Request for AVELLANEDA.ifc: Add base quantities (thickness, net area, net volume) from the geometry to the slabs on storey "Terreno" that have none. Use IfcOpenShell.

First a look at what the model holds.

```python
import ifcopenshell
import ifcopenshell.util.element
import ifcopenshell.util.unit

model = ifcopenshell.open("AVELLANEDA.ifc")
print(model.schema)
for unit_type in ("LENGTHUNIT", "AREAUNIT", "VOLUMEUNIT"):
    print(unit_type, ifcopenshell.util.unit.calculate_unit_scale(model, unit_type))
storey = next(s for s in model.by_type("IfcBuildingStorey") if s.Name == "Terreno")
slabs = [e for e in ifcopenshell.util.element.get_decomposition(storey) if e.is_a("IfcSlab")]
for e in sorted(slabs, key=lambda e: e.id()):
    print(e.id(), e.is_a(), e.Name, list(ifcopenshell.util.element.get_psets(e, qtos_only=True)), sep=" | ")
```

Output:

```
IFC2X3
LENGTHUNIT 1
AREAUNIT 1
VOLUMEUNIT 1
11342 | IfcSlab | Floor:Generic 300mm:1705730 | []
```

```python
import ifcopenshell
import ifcopenshell.api.pset
import ifcopenshell.geom
import ifcopenshell.util.element
import ifcopenshell.util.shape
import ifcopenshell.util.unit

model = ifcopenshell.open("AVELLANEDA.ifc")
unit_scale = ifcopenshell.util.unit.calculate_unit_scale(model)
area_scale = ifcopenshell.util.unit.calculate_unit_scale(model, "AREAUNIT")
volume_scale = ifcopenshell.util.unit.calculate_unit_scale(model, "VOLUMEUNIT")
settings = ifcopenshell.geom.settings()

storey = next(s for s in model.by_type("IfcBuildingStorey") if s.Name == "Terreno")
slabs = [e for e in ifcopenshell.util.element.get_decomposition(storey) if e.is_a("IfcSlab")]

for e in sorted(slabs, key=lambda e: e.id()):
    if ifcopenshell.util.element.get_psets(e, qtos_only=True, should_inherit=False):
        continue
    # Geometry comes back in metres, in the element's own axes.
    shape = ifcopenshell.geom.create_shape(settings, e)
    values = {
        "Width": ifcopenshell.util.shape.get_z(shape.geometry) / unit_scale,
        "NetArea": ifcopenshell.util.shape.get_footprint_area(shape.geometry) / area_scale,
        "NetVolume": ifcopenshell.util.shape.get_volume(shape.geometry) / volume_scale,
    }
    qto = ifcopenshell.api.pset.add_qto(model, product=e, name="BaseQuantities")
    ifcopenshell.api.pset.edit_qto(model, qto=qto, properties=values)
    print(e.id(), {k: round(v, 3) for k, v in values.items()})

model.write("AVELLANEDA-out.ifc")
```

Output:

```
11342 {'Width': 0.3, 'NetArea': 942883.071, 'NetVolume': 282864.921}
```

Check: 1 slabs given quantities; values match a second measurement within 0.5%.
